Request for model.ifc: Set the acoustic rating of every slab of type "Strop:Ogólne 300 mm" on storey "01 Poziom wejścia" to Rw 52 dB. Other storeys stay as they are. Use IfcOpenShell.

First a look at what the model holds.

```python
import ifcopenshell
import ifcopenshell.util.element

model = ifcopenshell.open("model.ifc")
print(model.schema)
storey = next(s for s in model.by_type("IfcBuildingStorey") if s.Name == "01 Poziom wejścia")
slabs = [e for e in ifcopenshell.util.element.get_decomposition(storey) if e.is_a("IfcSlab")]
seen = {}
for e in slabs:
    element_type = ifcopenshell.util.element.get_type(e)
    key = (element_type.Name if element_type != e and element_type else None, ifcopenshell.util.element.get_pset(e, "Pset_SlabCommon", "AcousticRating"))
    seen[key] = seen.get(key, 0) + 1
for (name, value), count in sorted(seen.items(), key=str):
    print(count, "x", name, "|", value)
```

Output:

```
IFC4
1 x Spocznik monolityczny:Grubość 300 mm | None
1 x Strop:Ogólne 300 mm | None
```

```python
import ifcopenshell
import ifcopenshell.api.pset
import ifcopenshell.util.element

model = ifcopenshell.open("model.ifc")

storey = next(s for s in model.by_type("IfcBuildingStorey") if s.Name == "01 Poziom wejścia")
slabs = [e for e in ifcopenshell.util.element.get_decomposition(storey) if e.is_a("IfcSlab")]

count = 0
for e in slabs:
    element_type = ifcopenshell.util.element.get_type(e)
    if element_type in (None, e) or element_type.Name != "Strop:Ogólne 300 mm":
        continue
    # add_pset returns the element's existing set when there is one.
    pset = ifcopenshell.api.pset.add_pset(model, product=e, name="Pset_SlabCommon")
    ifcopenshell.api.pset.edit_pset(model, pset=pset, properties={"AcousticRating": "Rw 52 dB"})
    count += 1

print(count, "slabs updated")

model.write("model_v2.ifc")
```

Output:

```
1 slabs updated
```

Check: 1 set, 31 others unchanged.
